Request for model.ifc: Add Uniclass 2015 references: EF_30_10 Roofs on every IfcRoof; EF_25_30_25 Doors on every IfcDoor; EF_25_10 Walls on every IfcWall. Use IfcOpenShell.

First a look at what the model holds.

```python
import ifcopenshell

model = ifcopenshell.open("model.ifc")
print(model.schema)
print("classifications:", [c.Name for c in model.by_type("IfcClassification")])
for ifc_class in ("IfcDoor", "IfcRoof", "IfcStair", "IfcWall", "IfcWindow"):
    print(ifc_class, len(model.by_type(ifc_class)))
```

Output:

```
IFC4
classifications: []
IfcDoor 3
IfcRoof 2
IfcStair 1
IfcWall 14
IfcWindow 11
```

```python
import ifcopenshell
import ifcopenshell.api.classification

model = ifcopenshell.open("model.ifc")

system = ifcopenshell.api.classification.add_classification(model, classification="Uniclass 2015")

codes = {
    "IfcRoof": ("EF_30_10", "Roofs"),
    "IfcDoor": ("EF_25_30_25", "Doors"),
    "IfcWall": ("EF_25_10", "Walls"),
}
for ifc_class, (code, name) in codes.items():
    products = model.by_type(ifc_class)
    ifcopenshell.api.classification.add_reference(
        model, products=products, classification=system, identification=code, name=name
    )
    print(code, len(products))

model.write("model_updated.ifc")
```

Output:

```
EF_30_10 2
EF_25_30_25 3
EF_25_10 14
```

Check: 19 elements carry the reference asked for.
